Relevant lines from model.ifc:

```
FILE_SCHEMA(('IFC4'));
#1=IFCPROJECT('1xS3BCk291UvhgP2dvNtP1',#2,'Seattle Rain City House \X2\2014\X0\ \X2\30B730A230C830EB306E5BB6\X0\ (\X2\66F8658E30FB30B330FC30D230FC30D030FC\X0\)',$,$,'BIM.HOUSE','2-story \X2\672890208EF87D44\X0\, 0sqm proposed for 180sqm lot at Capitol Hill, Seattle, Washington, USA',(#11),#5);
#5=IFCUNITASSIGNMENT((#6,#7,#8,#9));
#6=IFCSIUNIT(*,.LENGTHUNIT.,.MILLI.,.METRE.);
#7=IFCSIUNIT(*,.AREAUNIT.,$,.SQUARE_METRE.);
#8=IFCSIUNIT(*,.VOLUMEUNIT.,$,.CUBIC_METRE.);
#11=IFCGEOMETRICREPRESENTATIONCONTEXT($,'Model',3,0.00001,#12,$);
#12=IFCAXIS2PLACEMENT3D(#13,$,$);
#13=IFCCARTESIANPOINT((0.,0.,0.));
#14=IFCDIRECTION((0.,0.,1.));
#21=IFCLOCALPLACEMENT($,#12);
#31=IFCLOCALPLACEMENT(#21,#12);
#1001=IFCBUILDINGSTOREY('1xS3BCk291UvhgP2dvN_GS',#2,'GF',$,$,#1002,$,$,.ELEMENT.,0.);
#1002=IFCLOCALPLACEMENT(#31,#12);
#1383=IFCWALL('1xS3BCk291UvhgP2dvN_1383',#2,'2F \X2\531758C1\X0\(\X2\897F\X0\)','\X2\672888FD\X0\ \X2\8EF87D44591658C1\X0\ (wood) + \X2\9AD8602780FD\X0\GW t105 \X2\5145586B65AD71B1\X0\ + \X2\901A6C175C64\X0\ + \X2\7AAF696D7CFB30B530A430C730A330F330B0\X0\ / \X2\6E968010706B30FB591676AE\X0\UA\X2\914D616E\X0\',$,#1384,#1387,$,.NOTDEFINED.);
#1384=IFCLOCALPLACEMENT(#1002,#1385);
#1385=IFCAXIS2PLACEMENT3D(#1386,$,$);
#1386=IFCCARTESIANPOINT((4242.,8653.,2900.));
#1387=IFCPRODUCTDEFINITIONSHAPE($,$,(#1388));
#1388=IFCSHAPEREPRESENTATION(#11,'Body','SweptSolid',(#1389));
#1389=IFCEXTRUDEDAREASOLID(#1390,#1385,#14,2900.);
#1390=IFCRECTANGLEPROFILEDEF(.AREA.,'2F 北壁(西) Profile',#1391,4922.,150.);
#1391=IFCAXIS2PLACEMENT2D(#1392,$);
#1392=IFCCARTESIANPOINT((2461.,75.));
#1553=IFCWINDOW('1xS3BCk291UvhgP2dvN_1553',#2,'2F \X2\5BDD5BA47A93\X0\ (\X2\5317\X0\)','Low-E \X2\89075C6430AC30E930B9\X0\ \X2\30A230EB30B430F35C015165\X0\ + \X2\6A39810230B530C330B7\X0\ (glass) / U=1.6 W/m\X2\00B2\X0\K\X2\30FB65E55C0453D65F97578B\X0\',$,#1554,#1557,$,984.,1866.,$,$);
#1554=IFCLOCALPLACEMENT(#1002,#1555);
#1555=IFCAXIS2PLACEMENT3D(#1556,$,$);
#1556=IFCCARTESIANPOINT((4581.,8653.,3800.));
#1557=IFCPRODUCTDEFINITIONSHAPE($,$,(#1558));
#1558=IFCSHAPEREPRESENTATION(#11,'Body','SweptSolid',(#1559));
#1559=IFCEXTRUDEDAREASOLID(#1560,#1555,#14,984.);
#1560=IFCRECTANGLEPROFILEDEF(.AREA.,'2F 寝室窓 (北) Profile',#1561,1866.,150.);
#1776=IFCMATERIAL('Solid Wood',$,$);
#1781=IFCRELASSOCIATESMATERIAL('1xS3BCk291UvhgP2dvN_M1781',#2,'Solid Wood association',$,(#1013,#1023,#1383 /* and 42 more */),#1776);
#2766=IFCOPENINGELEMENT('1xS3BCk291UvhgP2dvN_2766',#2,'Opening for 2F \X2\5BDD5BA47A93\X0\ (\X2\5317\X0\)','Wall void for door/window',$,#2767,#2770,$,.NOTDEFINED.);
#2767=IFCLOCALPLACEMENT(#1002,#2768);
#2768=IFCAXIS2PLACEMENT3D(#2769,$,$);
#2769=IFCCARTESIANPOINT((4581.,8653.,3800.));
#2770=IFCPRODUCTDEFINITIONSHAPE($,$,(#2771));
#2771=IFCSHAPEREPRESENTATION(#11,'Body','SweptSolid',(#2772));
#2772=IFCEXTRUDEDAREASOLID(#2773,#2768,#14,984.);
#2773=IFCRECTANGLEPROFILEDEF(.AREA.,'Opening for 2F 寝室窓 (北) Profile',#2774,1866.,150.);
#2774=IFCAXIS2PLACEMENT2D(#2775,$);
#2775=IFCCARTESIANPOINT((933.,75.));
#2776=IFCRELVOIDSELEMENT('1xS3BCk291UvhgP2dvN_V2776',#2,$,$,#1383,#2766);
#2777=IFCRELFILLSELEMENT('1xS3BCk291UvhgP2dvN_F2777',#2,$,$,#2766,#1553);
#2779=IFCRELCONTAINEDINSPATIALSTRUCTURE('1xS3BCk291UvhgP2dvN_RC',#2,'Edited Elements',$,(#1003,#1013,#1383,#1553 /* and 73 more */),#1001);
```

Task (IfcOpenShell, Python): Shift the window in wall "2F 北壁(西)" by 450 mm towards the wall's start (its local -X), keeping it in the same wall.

```python
import ifcopenshell
import ifcopenshell.api.geometry
import ifcopenshell.util.placement
import ifcopenshell.util.unit

model = ifcopenshell.open("model.ifc")
unit_scale = ifcopenshell.util.unit.calculate_unit_scale(model)

window = model.by_id(1553)
opening = window.FillsVoids[0].RelatingOpeningElement
wall = opening.VoidsElements[0].RelatingBuildingElement

wall_matrix = ifcopenshell.util.placement.get_local_placement(wall.ObjectPlacement)
shift = wall_matrix[:3, 0] * -0.45 / unit_scale
before = ifcopenshell.util.placement.get_local_placement(window.ObjectPlacement)[:3, 3].copy()

# The window is not placed relative to its opening, so move both.
for product in (opening, window):
    matrix = ifcopenshell.util.placement.get_local_placement(product.ObjectPlacement)
    matrix[:3, 3] += shift
    ifcopenshell.api.geometry.edit_object_placement(model, product=product, matrix=matrix, is_si=False)

after = ifcopenshell.util.placement.get_local_placement(window.ObjectPlacement)[:3, 3]
print("window moved by", (after - before).round(3) + 0.0)

model.write("model_edited.ifc")
```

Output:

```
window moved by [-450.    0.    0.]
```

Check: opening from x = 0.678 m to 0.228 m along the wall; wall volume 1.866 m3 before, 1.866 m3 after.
